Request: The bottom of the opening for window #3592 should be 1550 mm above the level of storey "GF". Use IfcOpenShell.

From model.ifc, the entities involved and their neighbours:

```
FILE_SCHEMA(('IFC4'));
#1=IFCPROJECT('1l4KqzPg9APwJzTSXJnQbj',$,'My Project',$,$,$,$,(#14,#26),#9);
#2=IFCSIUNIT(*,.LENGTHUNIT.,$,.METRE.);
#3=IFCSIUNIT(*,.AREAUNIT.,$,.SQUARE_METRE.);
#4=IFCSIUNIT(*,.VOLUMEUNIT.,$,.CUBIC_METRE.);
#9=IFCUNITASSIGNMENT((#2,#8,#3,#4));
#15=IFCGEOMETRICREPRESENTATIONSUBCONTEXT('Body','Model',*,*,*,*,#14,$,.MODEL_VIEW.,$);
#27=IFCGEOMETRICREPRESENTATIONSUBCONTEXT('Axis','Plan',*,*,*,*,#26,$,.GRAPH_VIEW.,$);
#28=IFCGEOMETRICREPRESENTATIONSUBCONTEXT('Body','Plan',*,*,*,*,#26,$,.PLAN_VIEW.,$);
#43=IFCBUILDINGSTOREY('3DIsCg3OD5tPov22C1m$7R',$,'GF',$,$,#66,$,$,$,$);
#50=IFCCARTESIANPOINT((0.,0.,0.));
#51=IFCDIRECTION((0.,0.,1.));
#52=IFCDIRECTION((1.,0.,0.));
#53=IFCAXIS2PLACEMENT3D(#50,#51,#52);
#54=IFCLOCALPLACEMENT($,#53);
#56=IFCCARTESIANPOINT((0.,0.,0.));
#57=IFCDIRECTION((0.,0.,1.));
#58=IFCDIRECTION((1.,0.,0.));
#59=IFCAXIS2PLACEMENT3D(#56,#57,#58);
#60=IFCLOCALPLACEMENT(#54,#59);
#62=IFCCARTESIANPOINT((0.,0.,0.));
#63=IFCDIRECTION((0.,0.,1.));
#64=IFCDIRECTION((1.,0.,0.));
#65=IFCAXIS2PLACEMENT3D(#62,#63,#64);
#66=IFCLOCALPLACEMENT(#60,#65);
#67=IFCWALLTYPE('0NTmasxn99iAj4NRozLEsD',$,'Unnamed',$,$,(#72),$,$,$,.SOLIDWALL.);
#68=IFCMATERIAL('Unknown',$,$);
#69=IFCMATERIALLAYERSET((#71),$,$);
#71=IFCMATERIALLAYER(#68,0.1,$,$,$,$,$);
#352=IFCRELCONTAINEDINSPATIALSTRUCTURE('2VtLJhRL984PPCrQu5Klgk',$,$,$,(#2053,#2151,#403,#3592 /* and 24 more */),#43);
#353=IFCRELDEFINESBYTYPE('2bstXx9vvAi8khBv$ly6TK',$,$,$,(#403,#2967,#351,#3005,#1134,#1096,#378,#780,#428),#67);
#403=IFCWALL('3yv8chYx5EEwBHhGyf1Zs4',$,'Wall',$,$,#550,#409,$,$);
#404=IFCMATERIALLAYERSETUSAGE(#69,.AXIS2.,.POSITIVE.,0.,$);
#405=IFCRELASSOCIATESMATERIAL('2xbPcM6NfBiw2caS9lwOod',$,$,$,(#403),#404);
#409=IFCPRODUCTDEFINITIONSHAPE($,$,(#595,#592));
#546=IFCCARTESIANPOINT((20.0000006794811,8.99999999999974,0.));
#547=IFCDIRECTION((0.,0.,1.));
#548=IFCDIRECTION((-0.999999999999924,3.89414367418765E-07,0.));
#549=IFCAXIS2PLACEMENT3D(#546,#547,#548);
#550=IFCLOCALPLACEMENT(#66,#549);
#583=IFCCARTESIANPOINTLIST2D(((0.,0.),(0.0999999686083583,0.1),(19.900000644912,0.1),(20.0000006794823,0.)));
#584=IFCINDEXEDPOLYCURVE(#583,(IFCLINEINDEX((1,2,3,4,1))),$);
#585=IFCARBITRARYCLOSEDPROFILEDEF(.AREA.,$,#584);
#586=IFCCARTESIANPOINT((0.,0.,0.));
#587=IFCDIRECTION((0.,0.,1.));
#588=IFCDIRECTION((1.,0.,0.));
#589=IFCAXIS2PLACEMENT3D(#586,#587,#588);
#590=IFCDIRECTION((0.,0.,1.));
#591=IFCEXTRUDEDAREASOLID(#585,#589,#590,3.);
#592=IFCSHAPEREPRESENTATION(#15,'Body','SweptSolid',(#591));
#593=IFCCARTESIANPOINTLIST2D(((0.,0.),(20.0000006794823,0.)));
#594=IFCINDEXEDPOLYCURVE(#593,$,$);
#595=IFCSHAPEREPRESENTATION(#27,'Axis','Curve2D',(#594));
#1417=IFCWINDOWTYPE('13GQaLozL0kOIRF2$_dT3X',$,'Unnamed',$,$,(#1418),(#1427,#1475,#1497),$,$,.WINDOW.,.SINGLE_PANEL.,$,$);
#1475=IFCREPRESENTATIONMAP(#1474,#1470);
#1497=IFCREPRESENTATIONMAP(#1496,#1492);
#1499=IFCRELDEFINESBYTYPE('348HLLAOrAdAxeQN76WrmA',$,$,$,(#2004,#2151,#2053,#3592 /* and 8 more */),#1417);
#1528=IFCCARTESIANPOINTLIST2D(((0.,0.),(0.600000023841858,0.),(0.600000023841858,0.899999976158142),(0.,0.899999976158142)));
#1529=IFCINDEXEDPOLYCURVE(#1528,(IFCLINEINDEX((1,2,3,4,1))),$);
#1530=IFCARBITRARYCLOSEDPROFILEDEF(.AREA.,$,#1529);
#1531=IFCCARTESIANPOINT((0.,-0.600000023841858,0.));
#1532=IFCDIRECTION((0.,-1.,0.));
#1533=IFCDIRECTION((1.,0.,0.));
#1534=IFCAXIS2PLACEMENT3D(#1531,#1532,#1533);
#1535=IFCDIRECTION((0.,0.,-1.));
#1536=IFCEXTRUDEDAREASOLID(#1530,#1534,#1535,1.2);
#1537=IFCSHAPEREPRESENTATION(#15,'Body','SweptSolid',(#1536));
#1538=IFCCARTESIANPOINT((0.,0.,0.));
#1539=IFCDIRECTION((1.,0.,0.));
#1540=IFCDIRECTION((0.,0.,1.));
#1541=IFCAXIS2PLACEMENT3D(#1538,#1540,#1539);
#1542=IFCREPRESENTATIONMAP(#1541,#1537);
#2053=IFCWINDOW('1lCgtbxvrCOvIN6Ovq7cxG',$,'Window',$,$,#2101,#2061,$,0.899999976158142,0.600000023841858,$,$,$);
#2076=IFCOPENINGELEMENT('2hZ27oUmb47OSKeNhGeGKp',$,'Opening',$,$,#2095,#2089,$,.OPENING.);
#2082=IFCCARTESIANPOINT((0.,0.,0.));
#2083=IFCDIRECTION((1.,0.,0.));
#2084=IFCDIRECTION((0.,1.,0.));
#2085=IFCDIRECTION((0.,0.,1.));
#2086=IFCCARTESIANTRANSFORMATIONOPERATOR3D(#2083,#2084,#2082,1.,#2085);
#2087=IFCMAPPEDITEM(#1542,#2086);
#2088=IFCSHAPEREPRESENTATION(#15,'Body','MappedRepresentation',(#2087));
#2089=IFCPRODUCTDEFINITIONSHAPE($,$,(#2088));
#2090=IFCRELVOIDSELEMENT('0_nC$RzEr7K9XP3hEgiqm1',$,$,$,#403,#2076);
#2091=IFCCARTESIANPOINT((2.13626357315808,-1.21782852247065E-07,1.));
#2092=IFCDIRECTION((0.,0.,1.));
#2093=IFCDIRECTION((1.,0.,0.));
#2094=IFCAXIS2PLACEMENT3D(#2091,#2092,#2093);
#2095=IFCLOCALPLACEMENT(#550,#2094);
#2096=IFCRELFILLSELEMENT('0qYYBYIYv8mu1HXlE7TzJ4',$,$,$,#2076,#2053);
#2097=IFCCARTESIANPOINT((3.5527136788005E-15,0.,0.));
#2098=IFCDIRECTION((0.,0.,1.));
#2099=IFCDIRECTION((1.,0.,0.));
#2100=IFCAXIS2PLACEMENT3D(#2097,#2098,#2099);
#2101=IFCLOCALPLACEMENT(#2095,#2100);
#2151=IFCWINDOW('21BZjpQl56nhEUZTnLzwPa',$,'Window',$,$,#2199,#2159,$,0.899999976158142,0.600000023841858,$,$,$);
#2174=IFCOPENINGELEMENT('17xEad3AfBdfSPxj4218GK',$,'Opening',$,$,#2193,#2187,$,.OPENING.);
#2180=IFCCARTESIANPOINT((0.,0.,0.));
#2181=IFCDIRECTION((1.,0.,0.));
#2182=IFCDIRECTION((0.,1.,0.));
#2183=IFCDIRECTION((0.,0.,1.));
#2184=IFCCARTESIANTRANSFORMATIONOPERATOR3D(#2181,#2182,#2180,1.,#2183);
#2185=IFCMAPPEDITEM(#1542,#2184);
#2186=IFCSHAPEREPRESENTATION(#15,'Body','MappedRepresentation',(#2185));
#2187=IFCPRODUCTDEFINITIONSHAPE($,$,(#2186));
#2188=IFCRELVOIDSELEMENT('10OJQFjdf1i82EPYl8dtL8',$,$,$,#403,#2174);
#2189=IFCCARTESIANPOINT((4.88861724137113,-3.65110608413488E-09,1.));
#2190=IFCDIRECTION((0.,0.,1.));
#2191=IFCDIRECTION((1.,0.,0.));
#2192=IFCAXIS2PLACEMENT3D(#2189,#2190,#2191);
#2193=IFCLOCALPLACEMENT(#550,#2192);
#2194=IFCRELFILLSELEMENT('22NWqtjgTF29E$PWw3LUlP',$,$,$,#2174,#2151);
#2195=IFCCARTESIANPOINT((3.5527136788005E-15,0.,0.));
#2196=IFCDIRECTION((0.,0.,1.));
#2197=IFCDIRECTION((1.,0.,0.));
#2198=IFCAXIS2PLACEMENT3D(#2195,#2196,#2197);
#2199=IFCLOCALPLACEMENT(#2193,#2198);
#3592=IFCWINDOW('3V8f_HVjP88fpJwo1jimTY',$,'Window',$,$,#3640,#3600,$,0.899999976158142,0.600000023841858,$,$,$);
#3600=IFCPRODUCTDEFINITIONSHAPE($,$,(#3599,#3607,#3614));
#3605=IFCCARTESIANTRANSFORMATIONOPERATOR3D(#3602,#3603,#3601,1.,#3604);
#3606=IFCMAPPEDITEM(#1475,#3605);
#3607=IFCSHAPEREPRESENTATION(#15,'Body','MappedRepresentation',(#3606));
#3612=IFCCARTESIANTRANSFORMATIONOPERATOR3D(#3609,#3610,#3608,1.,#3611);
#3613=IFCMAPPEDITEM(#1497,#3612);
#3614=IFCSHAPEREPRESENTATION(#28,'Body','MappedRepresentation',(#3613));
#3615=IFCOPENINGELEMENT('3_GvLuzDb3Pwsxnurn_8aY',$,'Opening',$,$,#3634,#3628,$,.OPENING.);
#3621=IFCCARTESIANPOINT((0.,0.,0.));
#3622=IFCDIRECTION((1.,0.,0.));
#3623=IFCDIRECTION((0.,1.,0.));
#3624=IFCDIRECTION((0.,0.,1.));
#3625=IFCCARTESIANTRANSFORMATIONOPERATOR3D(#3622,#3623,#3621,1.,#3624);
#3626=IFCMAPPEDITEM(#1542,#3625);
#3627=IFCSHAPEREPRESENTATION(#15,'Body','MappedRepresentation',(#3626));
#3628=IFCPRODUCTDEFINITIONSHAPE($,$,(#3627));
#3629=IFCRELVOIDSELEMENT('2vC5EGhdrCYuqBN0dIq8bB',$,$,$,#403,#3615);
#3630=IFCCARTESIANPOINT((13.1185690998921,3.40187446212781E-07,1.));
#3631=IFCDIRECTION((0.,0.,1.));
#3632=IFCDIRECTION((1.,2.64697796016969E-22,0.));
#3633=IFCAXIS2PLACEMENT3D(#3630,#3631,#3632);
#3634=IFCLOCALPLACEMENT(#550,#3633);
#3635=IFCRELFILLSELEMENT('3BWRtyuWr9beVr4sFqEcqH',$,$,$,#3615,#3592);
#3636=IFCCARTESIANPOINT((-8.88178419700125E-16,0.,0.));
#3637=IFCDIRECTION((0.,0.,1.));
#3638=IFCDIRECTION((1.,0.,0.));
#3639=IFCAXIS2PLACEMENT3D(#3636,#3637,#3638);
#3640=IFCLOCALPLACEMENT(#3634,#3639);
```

```python
import numpy as np
import ifcopenshell
import ifcopenshell.api.geometry
import ifcopenshell.geom
import ifcopenshell.util.element
import ifcopenshell.util.placement
import ifcopenshell.util.shape
import ifcopenshell.util.unit

model = ifcopenshell.open("model.ifc")
unit_scale = ifcopenshell.util.unit.calculate_unit_scale(model)

window = model.by_guid("3V8f_HVjP88fpJwo1jimTY")
opening = window.FillsVoids[0].RelatingOpeningElement
storey = ifcopenshell.util.element.get_container(window, ifc_class="IfcBuildingStorey")
level = ifcopenshell.util.placement.get_local_placement(storey.ObjectPlacement)[2, 3]

# The opening's origin need not be at the sill, so measure its lowest point.
shape = ifcopenshell.geom.create_shape(ifcopenshell.geom.settings(), opening)
bottom = ifcopenshell.util.shape.get_shape_bottom_elevation(shape, shape.geometry) / unit_scale
dz = level + 1.55 - bottom

shift = np.array([0.0, 0.0, dz])
# The window is placed relative to its opening, so it follows when the opening moves.
matrix = ifcopenshell.util.placement.get_local_placement(opening.ObjectPlacement)
matrix[:3, 3] += shift
ifcopenshell.api.geometry.edit_object_placement(
    model, product=opening, matrix=matrix, is_si=False, should_transform_children=True
)

print(f"moved by {dz * unit_scale:+.3f} m")

model.write("model_edited.ifc")
```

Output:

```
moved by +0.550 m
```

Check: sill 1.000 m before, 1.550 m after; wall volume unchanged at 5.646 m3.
